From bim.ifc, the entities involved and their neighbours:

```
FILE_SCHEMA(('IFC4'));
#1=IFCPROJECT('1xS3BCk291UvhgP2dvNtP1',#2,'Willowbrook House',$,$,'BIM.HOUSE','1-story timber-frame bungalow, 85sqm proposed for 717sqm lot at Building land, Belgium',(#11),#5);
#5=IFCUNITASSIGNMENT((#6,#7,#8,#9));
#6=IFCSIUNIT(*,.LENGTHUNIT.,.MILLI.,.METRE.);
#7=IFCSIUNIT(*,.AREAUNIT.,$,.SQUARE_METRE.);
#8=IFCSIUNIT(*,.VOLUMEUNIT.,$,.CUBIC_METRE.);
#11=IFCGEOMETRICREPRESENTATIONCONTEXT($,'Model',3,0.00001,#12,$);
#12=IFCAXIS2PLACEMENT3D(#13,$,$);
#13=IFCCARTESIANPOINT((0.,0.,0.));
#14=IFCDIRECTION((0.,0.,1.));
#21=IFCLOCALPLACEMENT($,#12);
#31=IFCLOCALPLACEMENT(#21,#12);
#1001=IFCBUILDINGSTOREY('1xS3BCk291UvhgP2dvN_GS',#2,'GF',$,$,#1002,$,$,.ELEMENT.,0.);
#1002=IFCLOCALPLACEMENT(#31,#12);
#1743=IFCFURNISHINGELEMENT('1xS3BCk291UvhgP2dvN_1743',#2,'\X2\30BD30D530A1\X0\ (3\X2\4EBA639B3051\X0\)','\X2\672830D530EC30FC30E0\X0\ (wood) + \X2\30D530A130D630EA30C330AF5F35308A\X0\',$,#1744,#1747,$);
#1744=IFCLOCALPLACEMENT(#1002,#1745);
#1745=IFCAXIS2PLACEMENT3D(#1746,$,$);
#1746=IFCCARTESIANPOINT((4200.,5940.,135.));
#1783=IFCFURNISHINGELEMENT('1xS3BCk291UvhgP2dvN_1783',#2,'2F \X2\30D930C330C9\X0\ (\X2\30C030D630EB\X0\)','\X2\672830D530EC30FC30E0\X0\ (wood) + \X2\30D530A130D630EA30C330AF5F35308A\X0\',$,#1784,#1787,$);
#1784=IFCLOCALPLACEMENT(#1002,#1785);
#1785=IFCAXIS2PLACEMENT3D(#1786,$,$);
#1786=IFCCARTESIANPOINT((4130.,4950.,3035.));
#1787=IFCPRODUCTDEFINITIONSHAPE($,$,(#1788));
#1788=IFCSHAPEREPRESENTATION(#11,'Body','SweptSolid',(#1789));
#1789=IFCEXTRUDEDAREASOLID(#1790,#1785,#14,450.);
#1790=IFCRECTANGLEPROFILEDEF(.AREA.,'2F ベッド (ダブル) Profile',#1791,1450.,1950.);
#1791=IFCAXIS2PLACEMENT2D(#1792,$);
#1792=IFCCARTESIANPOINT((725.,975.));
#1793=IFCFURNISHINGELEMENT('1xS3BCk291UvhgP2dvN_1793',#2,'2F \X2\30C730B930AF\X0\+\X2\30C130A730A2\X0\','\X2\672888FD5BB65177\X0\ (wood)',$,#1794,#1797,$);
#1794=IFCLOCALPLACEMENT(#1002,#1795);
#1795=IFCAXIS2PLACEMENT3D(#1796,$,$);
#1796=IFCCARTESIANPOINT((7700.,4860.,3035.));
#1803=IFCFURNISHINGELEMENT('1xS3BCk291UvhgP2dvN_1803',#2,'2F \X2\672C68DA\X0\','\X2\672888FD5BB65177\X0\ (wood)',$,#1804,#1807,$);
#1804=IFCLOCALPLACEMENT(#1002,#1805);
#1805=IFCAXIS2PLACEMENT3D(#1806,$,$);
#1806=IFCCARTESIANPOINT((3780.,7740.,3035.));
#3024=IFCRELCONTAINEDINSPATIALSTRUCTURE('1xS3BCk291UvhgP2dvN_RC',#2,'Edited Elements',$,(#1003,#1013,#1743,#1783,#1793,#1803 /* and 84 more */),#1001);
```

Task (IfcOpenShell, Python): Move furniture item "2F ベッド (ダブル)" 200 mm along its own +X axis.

```python
import ifcopenshell
import ifcopenshell.api.geometry
import ifcopenshell.util.placement
import ifcopenshell.util.unit

model = ifcopenshell.open("bim.ifc")
unit_scale = ifcopenshell.util.unit.calculate_unit_scale(model)

item = model.by_guid("1xS3BCk291UvhgP2dvN_1783")
matrix = ifcopenshell.util.placement.get_local_placement(item.ObjectPlacement)
matrix[:3, 3] += matrix[:3, 0] * 0.2 / unit_scale
ifcopenshell.api.geometry.edit_object_placement(model, product=item, matrix=matrix, is_si=False)

print(ifcopenshell.util.placement.get_local_placement(item.ObjectPlacement).round(3) + 0.0)

model.write("bim_rev.ifc")
```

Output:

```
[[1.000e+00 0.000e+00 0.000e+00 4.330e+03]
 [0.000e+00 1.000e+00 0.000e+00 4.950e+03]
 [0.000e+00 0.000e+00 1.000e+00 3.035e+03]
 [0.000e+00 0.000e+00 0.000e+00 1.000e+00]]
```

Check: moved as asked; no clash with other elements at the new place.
